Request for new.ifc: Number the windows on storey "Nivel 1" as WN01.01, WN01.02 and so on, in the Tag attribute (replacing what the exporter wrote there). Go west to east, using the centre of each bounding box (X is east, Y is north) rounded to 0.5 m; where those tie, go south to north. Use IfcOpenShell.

First a look at what the model holds.

```python
import ifcopenshell
import ifcopenshell.util.element
import ifcopenshell.util.placement

model = ifcopenshell.open("new.ifc")
print(model.schema)
storey = next(s for s in model.by_type("IfcBuildingStorey") if s.Name == "Nivel 1")
windows = [e for e in ifcopenshell.util.element.get_decomposition(storey) if e.is_a("IfcWindow")]
for e in sorted(windows, key=lambda e: e.id()):
    origin = ifcopenshell.util.placement.get_local_placement(e.ObjectPlacement)[:3, 3]
    print(e.id(), e.Tag, e.Name, origin.round(2) + 0.0, sep=" | ")
```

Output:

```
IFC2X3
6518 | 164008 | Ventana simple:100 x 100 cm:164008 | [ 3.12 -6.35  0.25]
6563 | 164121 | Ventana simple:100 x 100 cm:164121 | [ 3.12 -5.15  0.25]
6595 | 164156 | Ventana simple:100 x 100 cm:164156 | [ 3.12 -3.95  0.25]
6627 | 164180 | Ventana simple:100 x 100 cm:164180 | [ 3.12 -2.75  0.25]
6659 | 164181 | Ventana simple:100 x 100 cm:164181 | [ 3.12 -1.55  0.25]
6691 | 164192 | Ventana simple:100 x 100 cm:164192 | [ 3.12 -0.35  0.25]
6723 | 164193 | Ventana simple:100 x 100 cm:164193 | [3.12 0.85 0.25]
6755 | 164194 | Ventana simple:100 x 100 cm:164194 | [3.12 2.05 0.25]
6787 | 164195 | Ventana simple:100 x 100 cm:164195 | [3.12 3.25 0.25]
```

```python
import ifcopenshell
import ifcopenshell.geom
import ifcopenshell.util.element
import ifcopenshell.util.shape

model = ifcopenshell.open("new.ifc")
settings = ifcopenshell.geom.settings()
settings.set("use-world-coords", True)


def centre(element):
    shape = ifcopenshell.geom.create_shape(settings, element)
    return ifcopenshell.util.shape.get_bbox_centroid(shape.geometry)


storey = next(s for s in model.by_type("IfcBuildingStorey") if s.Name == "Nivel 1")
windows = [e for e in ifcopenshell.util.element.get_decomposition(storey) if e.is_a("IfcWindow")]

# Insertion points can sit at a corner or the storey origin, so sort by the geometry (in metres).
centres = {e: centre(e) for e in windows}
windows.sort(key=lambda e: (round(centres[e][0] / 0.5), centres[e][1]))

for i, e in enumerate(windows, start=1):
    number = f"WN01.{i:02d}"
    e.Tag = number
    print(e.id(), number)

model.write("new_updated.ifc")
```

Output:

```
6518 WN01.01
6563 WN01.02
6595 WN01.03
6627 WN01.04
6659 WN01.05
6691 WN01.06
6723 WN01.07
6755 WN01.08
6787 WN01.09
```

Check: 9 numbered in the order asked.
